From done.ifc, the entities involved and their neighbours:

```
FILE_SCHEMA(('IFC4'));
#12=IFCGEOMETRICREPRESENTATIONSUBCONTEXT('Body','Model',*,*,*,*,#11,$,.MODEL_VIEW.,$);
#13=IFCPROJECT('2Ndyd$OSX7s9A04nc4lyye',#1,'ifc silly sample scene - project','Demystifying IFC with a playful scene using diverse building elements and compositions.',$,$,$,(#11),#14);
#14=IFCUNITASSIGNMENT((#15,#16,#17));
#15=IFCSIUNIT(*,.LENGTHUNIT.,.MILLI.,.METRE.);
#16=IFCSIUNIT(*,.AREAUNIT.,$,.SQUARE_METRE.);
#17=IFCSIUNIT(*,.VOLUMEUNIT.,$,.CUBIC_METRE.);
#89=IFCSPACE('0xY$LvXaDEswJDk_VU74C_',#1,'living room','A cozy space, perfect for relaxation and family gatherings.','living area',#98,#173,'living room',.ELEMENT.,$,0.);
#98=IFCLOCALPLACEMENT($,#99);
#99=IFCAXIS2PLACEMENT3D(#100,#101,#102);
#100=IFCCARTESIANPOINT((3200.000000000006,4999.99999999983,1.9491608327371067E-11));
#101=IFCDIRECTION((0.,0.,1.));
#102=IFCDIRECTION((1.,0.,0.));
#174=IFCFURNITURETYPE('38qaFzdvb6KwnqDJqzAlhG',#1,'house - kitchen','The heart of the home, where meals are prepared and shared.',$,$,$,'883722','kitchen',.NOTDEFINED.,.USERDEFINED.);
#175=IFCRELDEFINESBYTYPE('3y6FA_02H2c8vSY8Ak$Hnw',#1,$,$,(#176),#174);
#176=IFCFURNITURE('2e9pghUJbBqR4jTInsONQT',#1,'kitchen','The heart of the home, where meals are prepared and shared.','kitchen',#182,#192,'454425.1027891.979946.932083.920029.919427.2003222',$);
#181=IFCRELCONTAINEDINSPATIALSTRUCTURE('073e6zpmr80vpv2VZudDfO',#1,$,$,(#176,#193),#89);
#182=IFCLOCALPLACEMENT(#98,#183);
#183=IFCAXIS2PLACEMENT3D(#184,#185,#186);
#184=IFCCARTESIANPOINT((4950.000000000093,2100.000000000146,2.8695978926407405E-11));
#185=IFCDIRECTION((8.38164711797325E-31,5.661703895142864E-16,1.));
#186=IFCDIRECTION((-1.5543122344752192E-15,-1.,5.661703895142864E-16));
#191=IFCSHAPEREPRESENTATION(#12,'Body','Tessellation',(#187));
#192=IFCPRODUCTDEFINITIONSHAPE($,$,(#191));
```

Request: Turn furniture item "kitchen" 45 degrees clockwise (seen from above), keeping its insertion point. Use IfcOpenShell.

```python
import ifcopenshell
import ifcopenshell.api.geometry
import ifcopenshell.util.placement

model = ifcopenshell.open("done.ifc")

item = model.by_id(176)
matrix = ifcopenshell.util.placement.get_local_placement(item.ObjectPlacement)
matrix = matrix @ ifcopenshell.util.placement.rotation(-45, "Z")
ifcopenshell.api.geometry.edit_object_placement(model, product=item, matrix=matrix, is_si=False)

print(ifcopenshell.util.placement.get_local_placement(item.ObjectPlacement).round(3) + 0.0)

model.write("done_v2.ifc")
```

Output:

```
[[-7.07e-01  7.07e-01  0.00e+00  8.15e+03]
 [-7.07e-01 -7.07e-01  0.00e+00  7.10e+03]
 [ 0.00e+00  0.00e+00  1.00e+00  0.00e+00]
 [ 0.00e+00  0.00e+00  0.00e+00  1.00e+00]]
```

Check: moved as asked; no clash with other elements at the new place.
